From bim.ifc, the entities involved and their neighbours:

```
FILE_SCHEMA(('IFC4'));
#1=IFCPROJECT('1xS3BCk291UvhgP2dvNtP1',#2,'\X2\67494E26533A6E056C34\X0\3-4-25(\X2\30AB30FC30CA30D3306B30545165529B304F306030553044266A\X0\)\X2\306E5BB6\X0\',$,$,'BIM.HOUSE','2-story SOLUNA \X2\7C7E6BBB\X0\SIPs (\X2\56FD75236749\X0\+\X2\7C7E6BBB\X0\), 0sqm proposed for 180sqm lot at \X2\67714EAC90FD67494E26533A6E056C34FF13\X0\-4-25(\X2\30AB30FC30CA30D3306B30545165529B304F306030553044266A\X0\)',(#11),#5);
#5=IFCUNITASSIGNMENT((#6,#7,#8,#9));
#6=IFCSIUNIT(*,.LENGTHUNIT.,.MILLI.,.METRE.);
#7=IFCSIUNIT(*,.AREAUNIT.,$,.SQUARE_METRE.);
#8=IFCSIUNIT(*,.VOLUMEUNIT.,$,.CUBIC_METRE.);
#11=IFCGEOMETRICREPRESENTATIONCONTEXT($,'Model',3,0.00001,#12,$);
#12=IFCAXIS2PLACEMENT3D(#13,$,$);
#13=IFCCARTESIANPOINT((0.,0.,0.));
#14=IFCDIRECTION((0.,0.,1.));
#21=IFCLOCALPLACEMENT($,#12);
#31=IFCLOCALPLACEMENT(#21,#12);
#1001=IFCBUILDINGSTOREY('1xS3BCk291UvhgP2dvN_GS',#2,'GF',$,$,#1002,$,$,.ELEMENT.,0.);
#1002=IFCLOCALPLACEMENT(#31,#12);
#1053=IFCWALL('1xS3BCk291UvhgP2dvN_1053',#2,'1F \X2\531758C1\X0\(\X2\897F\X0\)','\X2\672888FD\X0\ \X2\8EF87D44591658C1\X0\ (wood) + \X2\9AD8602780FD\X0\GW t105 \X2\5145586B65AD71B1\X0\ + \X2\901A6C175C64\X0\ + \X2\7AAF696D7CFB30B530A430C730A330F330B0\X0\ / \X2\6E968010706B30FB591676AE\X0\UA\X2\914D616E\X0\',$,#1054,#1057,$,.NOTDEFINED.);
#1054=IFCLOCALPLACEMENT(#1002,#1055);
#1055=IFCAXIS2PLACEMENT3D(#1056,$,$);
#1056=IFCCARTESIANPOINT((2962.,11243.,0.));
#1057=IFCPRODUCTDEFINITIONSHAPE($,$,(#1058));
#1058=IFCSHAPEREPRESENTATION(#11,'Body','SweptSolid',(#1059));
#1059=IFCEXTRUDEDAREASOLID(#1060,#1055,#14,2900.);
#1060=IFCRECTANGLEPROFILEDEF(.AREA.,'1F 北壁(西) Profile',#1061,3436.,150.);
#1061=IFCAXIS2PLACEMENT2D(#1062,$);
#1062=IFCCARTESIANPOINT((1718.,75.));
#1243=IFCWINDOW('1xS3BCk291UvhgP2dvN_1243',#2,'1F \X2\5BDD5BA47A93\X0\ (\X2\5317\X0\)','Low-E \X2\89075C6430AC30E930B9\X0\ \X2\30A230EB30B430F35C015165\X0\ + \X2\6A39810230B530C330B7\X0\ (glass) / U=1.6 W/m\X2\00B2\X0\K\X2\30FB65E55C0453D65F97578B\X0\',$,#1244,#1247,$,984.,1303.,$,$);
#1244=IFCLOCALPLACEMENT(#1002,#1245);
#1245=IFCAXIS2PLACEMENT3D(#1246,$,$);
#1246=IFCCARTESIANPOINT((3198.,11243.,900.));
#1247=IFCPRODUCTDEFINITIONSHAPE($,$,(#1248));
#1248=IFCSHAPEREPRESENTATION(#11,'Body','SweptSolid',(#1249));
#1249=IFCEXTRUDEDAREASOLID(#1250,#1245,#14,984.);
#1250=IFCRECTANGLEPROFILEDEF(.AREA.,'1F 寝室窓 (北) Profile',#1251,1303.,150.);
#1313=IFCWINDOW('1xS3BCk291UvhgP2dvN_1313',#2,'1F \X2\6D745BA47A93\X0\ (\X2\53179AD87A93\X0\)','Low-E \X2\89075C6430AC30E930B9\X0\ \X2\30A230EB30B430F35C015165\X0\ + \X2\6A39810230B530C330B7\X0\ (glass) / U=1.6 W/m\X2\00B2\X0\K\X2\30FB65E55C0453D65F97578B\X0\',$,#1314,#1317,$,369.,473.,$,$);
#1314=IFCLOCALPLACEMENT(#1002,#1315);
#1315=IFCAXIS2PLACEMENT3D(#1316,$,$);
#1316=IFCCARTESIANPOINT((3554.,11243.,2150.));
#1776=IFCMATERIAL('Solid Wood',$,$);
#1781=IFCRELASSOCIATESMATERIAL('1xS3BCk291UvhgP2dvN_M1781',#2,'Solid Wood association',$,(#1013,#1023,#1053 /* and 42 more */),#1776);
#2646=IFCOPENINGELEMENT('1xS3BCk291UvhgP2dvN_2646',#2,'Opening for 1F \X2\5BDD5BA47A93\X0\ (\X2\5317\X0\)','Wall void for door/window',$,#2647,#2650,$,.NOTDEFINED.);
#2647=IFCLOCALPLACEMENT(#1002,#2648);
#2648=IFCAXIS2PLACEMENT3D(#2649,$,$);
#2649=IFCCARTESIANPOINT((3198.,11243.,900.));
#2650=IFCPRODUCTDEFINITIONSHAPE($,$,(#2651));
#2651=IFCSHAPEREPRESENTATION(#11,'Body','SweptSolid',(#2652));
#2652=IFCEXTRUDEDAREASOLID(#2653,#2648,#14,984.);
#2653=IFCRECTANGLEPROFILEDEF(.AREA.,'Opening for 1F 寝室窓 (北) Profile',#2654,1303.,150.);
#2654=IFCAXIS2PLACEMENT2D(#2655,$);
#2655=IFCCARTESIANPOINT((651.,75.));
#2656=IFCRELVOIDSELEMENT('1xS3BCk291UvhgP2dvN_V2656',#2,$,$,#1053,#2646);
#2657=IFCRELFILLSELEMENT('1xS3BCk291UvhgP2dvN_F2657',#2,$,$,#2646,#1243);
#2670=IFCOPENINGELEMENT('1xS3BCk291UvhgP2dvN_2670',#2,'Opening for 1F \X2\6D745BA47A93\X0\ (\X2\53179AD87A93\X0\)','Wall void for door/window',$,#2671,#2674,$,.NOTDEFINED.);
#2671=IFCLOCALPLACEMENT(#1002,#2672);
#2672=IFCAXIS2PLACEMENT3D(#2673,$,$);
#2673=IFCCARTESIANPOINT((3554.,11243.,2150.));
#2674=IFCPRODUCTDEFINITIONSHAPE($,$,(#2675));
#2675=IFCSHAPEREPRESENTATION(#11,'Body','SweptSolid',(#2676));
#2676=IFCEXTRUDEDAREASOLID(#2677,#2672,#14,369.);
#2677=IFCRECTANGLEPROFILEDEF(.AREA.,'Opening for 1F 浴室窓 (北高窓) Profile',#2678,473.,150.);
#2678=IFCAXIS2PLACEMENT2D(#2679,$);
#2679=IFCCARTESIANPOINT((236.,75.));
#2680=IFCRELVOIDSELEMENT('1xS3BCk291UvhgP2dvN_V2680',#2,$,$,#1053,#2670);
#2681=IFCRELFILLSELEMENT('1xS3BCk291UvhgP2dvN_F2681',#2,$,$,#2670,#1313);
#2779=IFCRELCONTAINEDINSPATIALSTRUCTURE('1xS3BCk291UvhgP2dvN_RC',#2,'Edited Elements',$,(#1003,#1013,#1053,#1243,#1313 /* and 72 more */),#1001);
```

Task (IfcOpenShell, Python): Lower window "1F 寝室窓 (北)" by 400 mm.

```python
import numpy as np
import ifcopenshell
import ifcopenshell.api.geometry
import ifcopenshell.util.placement
import ifcopenshell.util.unit

model = ifcopenshell.open("bim.ifc")
unit_scale = ifcopenshell.util.unit.calculate_unit_scale(model)

window = model.by_guid("1xS3BCk291UvhgP2dvN_1243")
opening = window.FillsVoids[0].RelatingOpeningElement
dz = -400.0

shift = np.array([0.0, 0.0, dz])
# The window is not placed relative to its opening, so move both.
for product in (opening, window):
    matrix = ifcopenshell.util.placement.get_local_placement(product.ObjectPlacement)
    matrix[:3, 3] += shift
    ifcopenshell.api.geometry.edit_object_placement(model, product=product, matrix=matrix, is_si=False)

print(f"moved by {dz * unit_scale:+.3f} m")

model.write("bim_rev.ifc")
```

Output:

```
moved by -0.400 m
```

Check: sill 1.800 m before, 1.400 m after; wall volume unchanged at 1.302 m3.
